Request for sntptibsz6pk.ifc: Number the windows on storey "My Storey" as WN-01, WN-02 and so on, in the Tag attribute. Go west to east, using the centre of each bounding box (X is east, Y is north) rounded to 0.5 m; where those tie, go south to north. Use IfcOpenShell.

First a look at what the model holds.

```python
import ifcopenshell
import ifcopenshell.util.element
import ifcopenshell.util.placement

model = ifcopenshell.open("sntptibsz6pk.ifc")
print(model.schema)
storey = next(s for s in model.by_type("IfcBuildingStorey") if s.Name == "My Storey")
windows = [e for e in ifcopenshell.util.element.get_decomposition(storey) if e.is_a("IfcWindow")]
for e in sorted(windows, key=lambda e: e.id()):
    origin = ifcopenshell.util.placement.get_local_placement(e.ObjectPlacement)[:3, 3]
    print(e.id(), e.Tag, e.Name, origin.round(2) + 0.0, sep=" | ")
```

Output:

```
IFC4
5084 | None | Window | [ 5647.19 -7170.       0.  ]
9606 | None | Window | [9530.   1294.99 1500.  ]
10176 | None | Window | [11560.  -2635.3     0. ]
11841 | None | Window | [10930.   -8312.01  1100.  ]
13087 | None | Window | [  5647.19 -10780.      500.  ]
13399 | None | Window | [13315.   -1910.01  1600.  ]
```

```python
import ifcopenshell
import ifcopenshell.geom
import ifcopenshell.util.element
import ifcopenshell.util.shape

model = ifcopenshell.open("sntptibsz6pk.ifc")
settings = ifcopenshell.geom.settings()
settings.set("use-world-coords", True)


def centre(element):
    shape = ifcopenshell.geom.create_shape(settings, element)
    return ifcopenshell.util.shape.get_bbox_centroid(shape.geometry)


storey = next(s for s in model.by_type("IfcBuildingStorey") if s.Name == "My Storey")
windows = [e for e in ifcopenshell.util.element.get_decomposition(storey) if e.is_a("IfcWindow")]

# Insertion points can sit at a corner or the storey origin, so sort by the geometry (in metres).
centres = {e: centre(e) for e in windows}
windows.sort(key=lambda e: (round(centres[e][0] / 0.5), centres[e][1]))

for i, e in enumerate(windows, start=1):
    number = f"WN-{i:02d}"
    e.Tag = number
    print(e.id(), number)

model.write("sntptibsz6pk_v2.ifc")
```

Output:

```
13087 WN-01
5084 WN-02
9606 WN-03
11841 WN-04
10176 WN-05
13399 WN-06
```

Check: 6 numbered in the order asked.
